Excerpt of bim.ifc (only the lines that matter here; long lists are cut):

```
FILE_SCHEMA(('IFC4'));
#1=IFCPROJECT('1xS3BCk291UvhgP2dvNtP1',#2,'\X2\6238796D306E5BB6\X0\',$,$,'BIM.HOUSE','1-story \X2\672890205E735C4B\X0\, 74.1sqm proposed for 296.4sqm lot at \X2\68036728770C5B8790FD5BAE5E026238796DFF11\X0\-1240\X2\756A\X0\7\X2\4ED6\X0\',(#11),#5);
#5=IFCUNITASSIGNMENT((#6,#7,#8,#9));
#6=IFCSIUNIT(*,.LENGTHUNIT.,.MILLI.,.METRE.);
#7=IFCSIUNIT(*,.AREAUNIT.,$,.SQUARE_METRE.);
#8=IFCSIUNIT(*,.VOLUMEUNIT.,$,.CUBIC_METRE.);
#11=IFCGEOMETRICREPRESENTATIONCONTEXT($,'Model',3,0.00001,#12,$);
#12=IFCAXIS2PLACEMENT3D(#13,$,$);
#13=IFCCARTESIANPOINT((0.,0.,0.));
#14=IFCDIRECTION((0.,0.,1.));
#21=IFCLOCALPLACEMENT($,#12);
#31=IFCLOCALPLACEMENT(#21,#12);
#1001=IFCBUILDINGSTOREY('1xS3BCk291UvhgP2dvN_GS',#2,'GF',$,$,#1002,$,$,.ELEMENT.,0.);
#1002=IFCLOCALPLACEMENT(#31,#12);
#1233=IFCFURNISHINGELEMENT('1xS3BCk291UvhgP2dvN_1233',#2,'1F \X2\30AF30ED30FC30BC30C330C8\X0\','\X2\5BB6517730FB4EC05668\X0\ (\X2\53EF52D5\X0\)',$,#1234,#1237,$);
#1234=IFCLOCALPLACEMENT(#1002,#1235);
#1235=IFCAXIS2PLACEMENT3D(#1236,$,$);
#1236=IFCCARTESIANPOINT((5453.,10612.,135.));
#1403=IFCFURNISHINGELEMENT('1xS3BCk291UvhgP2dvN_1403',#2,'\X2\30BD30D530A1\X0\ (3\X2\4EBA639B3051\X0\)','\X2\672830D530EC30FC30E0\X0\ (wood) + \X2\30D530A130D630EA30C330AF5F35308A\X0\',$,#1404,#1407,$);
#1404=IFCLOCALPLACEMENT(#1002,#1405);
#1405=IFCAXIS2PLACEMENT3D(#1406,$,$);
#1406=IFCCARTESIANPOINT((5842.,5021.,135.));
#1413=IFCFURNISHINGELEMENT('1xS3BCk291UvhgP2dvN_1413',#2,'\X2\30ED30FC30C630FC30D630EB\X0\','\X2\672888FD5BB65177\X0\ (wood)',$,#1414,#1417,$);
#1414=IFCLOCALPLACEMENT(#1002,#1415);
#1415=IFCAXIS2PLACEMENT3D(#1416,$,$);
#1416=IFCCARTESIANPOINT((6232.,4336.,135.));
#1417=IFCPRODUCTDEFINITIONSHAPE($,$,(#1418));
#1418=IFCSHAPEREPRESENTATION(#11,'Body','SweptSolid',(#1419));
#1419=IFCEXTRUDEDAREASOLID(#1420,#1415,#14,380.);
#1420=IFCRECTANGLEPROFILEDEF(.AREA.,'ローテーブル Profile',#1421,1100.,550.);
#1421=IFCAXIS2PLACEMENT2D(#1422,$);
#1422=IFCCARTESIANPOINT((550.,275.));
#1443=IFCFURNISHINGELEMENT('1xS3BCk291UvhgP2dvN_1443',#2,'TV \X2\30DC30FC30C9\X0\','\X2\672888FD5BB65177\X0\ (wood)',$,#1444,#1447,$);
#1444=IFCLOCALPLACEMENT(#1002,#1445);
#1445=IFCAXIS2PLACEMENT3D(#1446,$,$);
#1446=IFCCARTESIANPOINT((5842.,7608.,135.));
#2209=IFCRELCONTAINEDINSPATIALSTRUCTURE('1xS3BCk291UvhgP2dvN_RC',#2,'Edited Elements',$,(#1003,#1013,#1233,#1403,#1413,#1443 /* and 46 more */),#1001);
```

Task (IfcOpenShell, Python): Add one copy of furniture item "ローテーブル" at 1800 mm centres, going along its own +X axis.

```python
import ifcopenshell
import ifcopenshell.api.geometry
import ifcopenshell.api.root
import ifcopenshell.util.element
import ifcopenshell.util.placement
import ifcopenshell.util.unit

model = ifcopenshell.open("bim.ifc")
unit_scale = ifcopenshell.util.unit.calculate_unit_scale(model)


def reuse_history(source, copy):
    """copy_class also copies each property set's owner history, people and application; keep the originals."""
    for rel in copy.IsDefinedBy:
        if rel.is_a("IfcRelDefinesByProperties") and (history := rel.RelatingPropertyDefinition.OwnerHistory):
            rel.RelatingPropertyDefinition.OwnerHistory = source.OwnerHistory
            ifcopenshell.util.element.remove_deep2(model, history)


source = model.by_id(1413)
base = ifcopenshell.util.placement.get_local_placement(source.ObjectPlacement)
step = base[:3, 0] * 1.8 / unit_scale

for i in range(1, 2):
    copy = ifcopenshell.api.root.copy_class(model, product=source)
    copy.Representation = ifcopenshell.util.element.copy_deep(
        model, source.Representation, exclude=["IfcGeometricRepresentationContext", "IfcRepresentationMap"]
    )
    reuse_history(source, copy)
    matrix = base.copy()
    matrix[:3, 3] += i * step
    print("added at", matrix[:3, 3].round(3) + 0.0)
    ifcopenshell.api.geometry.edit_object_placement(model, product=copy, matrix=matrix, is_si=False)

model.write("bim_v2.ifc")
```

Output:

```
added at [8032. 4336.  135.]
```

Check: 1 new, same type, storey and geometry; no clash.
